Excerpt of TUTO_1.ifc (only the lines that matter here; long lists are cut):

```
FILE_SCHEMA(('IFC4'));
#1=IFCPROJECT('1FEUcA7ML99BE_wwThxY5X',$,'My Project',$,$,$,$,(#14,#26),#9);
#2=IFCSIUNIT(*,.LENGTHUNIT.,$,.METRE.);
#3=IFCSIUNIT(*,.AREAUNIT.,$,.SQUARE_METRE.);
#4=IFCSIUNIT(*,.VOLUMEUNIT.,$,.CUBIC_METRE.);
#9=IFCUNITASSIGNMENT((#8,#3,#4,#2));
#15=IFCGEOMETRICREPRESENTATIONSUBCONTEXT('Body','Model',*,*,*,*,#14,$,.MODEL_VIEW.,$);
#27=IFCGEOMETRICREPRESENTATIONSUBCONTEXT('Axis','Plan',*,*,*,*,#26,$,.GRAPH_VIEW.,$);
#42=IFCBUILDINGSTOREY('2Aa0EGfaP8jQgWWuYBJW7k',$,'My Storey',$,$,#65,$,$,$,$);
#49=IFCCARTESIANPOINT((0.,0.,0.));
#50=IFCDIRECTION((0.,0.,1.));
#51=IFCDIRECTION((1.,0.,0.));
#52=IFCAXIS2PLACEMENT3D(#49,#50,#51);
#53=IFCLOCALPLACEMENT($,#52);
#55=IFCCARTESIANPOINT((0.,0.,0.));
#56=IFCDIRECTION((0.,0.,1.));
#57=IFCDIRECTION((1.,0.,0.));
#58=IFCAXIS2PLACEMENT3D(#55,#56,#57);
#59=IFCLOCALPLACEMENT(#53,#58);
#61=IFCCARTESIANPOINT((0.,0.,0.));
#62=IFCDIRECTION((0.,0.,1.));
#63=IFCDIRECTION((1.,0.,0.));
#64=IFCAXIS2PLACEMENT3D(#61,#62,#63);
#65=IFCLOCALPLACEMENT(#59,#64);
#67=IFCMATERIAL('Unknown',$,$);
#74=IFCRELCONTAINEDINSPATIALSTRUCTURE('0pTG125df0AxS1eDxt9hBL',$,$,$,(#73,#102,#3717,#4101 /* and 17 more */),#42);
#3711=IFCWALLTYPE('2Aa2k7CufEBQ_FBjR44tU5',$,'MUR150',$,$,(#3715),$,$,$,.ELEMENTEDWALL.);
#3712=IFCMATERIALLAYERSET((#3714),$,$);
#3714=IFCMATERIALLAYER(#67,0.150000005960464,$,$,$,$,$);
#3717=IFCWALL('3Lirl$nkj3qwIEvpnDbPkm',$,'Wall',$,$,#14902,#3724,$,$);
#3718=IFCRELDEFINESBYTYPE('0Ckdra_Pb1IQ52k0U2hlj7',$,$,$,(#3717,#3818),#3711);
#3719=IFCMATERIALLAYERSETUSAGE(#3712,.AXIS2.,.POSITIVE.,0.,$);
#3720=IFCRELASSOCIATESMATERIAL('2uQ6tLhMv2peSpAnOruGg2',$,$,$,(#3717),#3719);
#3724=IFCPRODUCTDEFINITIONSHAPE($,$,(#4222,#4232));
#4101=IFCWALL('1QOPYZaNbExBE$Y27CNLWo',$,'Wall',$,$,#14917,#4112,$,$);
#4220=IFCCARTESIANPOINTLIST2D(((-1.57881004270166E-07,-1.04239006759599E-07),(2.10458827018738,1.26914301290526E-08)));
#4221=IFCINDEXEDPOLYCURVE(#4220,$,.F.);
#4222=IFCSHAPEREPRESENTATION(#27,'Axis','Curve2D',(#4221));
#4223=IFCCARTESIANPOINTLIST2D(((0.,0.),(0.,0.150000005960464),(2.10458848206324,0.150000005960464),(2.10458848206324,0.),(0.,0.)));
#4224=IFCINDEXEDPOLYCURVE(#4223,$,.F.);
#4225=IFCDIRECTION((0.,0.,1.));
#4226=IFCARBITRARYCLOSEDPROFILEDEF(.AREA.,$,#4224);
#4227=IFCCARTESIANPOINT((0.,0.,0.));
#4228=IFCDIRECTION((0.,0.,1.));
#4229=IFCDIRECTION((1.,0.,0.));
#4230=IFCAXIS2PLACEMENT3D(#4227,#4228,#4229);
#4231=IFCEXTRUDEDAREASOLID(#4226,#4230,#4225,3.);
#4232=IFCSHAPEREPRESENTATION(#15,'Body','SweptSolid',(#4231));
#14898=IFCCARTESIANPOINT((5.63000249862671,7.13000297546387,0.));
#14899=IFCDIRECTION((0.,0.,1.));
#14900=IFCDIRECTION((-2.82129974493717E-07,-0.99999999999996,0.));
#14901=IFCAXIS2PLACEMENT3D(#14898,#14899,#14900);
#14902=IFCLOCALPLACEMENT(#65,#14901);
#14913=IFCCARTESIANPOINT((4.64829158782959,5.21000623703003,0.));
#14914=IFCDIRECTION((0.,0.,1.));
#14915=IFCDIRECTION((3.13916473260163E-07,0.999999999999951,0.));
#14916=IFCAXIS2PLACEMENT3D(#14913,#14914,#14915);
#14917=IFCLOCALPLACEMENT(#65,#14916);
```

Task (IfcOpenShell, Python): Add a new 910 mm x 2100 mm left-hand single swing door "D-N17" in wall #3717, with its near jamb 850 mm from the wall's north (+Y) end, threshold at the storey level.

```python
import numpy as np
import ifcopenshell
import ifcopenshell.api.feature
import ifcopenshell.api.geometry
import ifcopenshell.api.root
import ifcopenshell.api.spatial
import ifcopenshell.geom
import ifcopenshell.util.element
import ifcopenshell.util.placement
import ifcopenshell.util.representation
import ifcopenshell.util.shape
import ifcopenshell.util.unit

model = ifcopenshell.open("TUTO_1.ifc")
unit_scale = ifcopenshell.util.unit.calculate_unit_scale(model)
settings = ifcopenshell.geom.settings()


def volume(element):
    """Net volume in cubic metres, openings subtracted."""
    shape = ifcopenshell.geom.create_shape(settings, element)
    return ifcopenshell.util.shape.get_volume(shape.geometry)


wall = model.by_guid("3Lirl$nkj3qwIEvpnDbPkm")
storey = ifcopenshell.util.element.get_container(wall, ifc_class="IfcBuildingStorey")
context = ifcopenshell.util.representation.get_context(model, "Model", "Body", "MODEL_VIEW")
before = volume(wall)

width, height, from_end, sill = 0.91, 2.1, 0.85, 0.0  # metres

# The wall runs along its own X axis, and the end named is its -X end.
wall_shape = ifcopenshell.geom.create_shape(settings, wall)
x, y, z = ifcopenshell.util.shape.get_vertices(wall_shape.geometry).T
start = x.min() + from_end
face, thickness = float(y.min()), float(y.max() - y.min())
wall_matrix = ifcopenshell.util.placement.get_local_placement(wall.ObjectPlacement)
level = ifcopenshell.util.placement.get_local_placement(storey.ObjectPlacement)[2, 3]


def in_wall(x, y):
    """Placement at x, y metres in the wall's axes, at sill height."""
    matrix = wall_matrix.copy()
    matrix[:, 3] = wall_matrix @ np.array([x / unit_scale, y / unit_scale, 0.0, 1.0])
    matrix[2, 3] = level + sill / unit_scale
    return matrix


# Opening: a box that overshoots both wall faces by 50 mm.
opening = ifcopenshell.api.root.create_entity(model, ifc_class="IfcOpeningElement", predefined_type="OPENING")
box = ifcopenshell.api.geometry.add_wall_representation(
    model, context=context, length=width, height=height, thickness=thickness + 0.1
)
ifcopenshell.api.geometry.assign_representation(model, product=opening, representation=box)
ifcopenshell.api.geometry.edit_object_placement(model, product=opening, matrix=in_wall(start, face - 0.05), is_si=False)
ifcopenshell.api.feature.add_feature(model, feature=opening, element=wall)

door = ifcopenshell.api.root.create_entity(model, ifc_class="IfcDoor", name="D-N17", predefined_type="DOOR")
door.OverallWidth, door.OverallHeight = width / unit_scale, height / unit_scale
door.OperationType = "SINGLE_SWING_LEFT"
body = ifcopenshell.api.geometry.add_door_representation(
    model,
    context=context,
    overall_width=door.OverallWidth,
    overall_height=door.OverallHeight,
    operation_type="SINGLE_SWING_LEFT",
    lining_properties={"LiningDepth": thickness / unit_scale, "ThresholdDepth": thickness / unit_scale},
)
ifcopenshell.api.geometry.assign_representation(model, product=door, representation=body)
ifcopenshell.api.spatial.assign_container(model, products=[door], relating_structure=storey)
ifcopenshell.api.feature.add_filling(model, opening=opening, element=door)

# The lining spans the wall, so the door starts at the wall face.
ifcopenshell.api.geometry.edit_object_placement(model, product=door, matrix=in_wall(start, face), is_si=False)

after = volume(wall)

print(f"wall volume {before:.3f} -> {after:.3f} m3")

model.write("TUTO_1-out.ifc")
```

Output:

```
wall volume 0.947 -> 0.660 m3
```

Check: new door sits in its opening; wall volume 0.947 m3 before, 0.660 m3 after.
